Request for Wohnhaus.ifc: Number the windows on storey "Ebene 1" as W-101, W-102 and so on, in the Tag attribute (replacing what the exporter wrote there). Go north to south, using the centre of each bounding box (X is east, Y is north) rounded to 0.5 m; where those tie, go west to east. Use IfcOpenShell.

First a look at what the model holds.

```python
import ifcopenshell
import ifcopenshell.util.element
import ifcopenshell.util.placement

model = ifcopenshell.open("Wohnhaus.ifc")
print(model.schema)
storey = next(s for s in model.by_type("IfcBuildingStorey") if s.Name == "Ebene 1")
windows = [e for e in ifcopenshell.util.element.get_decomposition(storey) if e.is_a("IfcWindow")]
for e in sorted(windows, key=lambda e: e.id()):
    origin = ifcopenshell.util.placement.get_local_placement(e.ObjectPlacement)[:3, 3]
    print(e.id(), e.Tag, e.Name, origin.round(2) + 0.0, sep=" | ")
```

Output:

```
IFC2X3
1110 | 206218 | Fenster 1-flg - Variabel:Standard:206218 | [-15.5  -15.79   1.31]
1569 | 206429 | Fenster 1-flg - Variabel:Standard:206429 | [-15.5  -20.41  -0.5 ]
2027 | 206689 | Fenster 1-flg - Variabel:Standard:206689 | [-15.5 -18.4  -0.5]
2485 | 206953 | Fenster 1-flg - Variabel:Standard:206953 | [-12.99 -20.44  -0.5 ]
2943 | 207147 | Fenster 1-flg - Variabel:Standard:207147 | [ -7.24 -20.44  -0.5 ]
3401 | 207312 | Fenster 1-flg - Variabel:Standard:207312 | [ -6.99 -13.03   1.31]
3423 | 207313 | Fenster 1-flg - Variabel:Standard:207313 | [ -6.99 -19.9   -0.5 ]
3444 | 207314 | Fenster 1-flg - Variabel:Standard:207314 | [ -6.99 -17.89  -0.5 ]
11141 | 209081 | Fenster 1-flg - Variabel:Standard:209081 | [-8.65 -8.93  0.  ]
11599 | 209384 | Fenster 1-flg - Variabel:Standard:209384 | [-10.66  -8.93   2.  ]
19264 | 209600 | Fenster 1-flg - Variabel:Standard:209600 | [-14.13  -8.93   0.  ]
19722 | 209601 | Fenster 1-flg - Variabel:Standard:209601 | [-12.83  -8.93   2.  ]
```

```python
import ifcopenshell
import ifcopenshell.geom
import ifcopenshell.util.element
import ifcopenshell.util.shape

model = ifcopenshell.open("Wohnhaus.ifc")
settings = ifcopenshell.geom.settings()
settings.set("use-world-coords", True)


def centre(element):
    shape = ifcopenshell.geom.create_shape(settings, element)
    return ifcopenshell.util.shape.get_bbox_centroid(shape.geometry)


storey = next(s for s in model.by_type("IfcBuildingStorey") if s.Name == "Ebene 1")
windows = [e for e in ifcopenshell.util.element.get_decomposition(storey) if e.is_a("IfcWindow")]

# Insertion points can sit at a corner or the storey origin, so sort by the geometry (in metres).
centres = {e: centre(e) for e in windows}
windows.sort(key=lambda e: (-round(centres[e][1] / 0.5), centres[e][0]))

for i, e in enumerate(windows, start=1):
    number = f"W-1{i:02d}"
    e.Tag = number
    print(e.id(), number)

model.write("Wohnhaus_v2.ifc")
```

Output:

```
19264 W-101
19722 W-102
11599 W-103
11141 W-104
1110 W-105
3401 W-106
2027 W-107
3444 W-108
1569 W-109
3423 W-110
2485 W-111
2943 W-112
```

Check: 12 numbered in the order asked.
